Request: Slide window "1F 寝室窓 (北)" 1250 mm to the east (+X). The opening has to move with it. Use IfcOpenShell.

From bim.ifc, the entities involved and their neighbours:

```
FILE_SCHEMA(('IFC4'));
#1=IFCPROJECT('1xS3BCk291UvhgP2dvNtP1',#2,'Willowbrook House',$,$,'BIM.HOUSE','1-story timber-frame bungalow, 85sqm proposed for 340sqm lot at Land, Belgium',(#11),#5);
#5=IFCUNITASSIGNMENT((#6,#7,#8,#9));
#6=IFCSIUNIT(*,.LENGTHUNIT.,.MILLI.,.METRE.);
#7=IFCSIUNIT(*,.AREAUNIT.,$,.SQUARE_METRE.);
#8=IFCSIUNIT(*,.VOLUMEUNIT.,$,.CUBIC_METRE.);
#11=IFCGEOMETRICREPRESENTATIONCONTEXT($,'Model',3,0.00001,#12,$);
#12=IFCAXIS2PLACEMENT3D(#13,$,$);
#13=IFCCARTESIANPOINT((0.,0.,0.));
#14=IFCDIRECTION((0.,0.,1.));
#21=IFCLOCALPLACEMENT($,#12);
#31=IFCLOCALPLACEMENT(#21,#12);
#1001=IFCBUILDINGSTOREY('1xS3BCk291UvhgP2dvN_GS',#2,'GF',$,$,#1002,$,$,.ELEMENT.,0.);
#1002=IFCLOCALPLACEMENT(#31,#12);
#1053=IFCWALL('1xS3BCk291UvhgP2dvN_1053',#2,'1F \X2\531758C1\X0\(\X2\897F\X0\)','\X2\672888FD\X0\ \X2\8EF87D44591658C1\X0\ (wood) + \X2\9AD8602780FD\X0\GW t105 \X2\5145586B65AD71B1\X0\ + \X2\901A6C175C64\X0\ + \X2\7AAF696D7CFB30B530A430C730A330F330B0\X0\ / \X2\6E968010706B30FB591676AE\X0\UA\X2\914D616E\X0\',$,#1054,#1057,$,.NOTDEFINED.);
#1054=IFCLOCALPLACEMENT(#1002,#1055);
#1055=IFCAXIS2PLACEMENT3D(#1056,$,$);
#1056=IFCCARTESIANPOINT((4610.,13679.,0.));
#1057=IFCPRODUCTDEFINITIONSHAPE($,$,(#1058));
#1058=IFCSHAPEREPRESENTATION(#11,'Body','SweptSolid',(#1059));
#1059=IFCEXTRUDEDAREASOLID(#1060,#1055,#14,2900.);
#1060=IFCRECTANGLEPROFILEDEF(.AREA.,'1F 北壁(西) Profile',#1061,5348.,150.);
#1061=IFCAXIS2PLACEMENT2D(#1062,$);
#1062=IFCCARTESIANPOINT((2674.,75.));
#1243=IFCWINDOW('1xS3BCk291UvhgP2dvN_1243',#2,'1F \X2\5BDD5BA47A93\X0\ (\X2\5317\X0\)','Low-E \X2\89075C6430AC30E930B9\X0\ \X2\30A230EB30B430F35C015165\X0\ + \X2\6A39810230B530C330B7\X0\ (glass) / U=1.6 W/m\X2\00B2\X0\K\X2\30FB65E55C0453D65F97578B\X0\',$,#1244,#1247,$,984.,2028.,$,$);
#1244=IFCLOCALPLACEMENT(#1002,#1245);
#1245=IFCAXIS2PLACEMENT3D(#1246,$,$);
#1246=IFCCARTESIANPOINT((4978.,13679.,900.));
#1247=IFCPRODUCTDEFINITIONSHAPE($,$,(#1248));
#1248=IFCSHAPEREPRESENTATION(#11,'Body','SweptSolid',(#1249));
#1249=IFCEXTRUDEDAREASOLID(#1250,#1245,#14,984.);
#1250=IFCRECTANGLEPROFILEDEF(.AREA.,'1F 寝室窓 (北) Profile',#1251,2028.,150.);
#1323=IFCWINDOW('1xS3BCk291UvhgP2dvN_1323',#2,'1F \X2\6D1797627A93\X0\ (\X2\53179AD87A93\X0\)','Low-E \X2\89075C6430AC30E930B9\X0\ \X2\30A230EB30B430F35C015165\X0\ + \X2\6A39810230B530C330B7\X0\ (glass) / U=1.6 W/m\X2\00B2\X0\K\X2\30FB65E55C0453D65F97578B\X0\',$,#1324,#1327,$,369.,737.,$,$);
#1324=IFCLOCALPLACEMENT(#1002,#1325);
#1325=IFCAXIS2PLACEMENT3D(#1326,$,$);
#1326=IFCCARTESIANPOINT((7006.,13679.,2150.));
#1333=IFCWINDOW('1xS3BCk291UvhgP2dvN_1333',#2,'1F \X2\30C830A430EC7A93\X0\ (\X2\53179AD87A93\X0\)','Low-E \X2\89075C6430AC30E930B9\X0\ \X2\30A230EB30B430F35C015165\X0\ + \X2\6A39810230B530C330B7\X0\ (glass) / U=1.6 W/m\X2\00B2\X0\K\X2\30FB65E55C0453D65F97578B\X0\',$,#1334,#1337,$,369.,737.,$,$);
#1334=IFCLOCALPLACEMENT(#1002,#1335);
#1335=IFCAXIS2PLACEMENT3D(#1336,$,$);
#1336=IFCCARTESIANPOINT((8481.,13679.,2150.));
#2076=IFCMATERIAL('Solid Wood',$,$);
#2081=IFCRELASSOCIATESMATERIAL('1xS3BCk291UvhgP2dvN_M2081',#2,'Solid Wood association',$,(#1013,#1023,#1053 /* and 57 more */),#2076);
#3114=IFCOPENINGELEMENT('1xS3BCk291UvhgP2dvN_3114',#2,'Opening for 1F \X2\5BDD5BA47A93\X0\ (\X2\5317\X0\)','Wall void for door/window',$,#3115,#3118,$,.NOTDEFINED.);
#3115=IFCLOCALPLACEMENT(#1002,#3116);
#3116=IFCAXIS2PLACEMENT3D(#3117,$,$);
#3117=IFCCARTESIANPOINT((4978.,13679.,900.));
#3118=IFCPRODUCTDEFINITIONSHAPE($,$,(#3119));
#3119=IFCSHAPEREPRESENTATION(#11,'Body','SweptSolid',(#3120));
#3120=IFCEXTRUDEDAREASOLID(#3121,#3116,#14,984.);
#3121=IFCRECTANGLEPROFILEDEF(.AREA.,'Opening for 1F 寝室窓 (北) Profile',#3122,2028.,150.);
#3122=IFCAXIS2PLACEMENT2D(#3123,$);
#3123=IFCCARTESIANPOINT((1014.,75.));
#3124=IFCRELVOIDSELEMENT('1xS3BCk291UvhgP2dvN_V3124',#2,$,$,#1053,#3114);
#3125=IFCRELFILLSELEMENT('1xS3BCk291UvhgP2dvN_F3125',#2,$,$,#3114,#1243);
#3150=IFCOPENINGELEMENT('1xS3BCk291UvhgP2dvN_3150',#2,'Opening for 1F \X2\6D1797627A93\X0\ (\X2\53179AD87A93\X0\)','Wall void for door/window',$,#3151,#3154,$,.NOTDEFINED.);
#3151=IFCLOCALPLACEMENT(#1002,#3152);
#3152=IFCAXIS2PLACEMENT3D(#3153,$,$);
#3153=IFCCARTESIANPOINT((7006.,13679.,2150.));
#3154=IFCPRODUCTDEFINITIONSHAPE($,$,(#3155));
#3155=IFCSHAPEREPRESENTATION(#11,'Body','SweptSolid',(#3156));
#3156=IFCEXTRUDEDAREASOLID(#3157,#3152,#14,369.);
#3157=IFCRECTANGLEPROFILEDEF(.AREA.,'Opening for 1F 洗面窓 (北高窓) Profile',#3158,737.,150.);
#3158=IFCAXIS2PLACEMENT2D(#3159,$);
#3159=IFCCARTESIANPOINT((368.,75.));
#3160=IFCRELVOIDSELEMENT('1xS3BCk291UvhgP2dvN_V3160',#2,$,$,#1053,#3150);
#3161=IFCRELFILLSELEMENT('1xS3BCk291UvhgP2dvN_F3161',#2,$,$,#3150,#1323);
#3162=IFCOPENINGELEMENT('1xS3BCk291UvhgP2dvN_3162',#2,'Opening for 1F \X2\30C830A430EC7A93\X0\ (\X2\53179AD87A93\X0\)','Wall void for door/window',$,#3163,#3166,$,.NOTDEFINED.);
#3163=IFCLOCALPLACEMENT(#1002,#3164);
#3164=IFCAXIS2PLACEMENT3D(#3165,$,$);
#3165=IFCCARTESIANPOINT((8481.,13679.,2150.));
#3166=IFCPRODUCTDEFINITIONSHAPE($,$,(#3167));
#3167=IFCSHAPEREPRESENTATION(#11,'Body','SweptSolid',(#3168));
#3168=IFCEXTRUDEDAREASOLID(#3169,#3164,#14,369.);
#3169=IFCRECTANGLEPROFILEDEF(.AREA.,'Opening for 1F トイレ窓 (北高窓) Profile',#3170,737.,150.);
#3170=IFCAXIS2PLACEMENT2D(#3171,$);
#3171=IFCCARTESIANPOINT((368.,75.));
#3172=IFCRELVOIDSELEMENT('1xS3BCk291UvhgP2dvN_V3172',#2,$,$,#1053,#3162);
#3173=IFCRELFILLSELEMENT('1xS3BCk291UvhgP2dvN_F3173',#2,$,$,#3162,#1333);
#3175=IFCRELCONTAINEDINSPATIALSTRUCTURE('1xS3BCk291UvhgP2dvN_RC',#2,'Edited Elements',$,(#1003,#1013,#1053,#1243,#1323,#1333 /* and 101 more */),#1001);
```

```python
import ifcopenshell
import ifcopenshell.api.geometry
import ifcopenshell.util.placement

model = ifcopenshell.open("bim.ifc")

window = model.by_id(1243)
opening = window.FillsVoids[0].RelatingOpeningElement
wall = opening.VoidsElements[0].RelatingBuildingElement

wall_matrix = ifcopenshell.util.placement.get_local_placement(wall.ObjectPlacement)
shift = wall_matrix[:3, 0] * 1250.0
before = ifcopenshell.util.placement.get_local_placement(window.ObjectPlacement)[:3, 3].copy()

# The window is not placed relative to its opening, so move both.
for product in (opening, window):
    matrix = ifcopenshell.util.placement.get_local_placement(product.ObjectPlacement)
    matrix[:3, 3] += shift
    ifcopenshell.api.geometry.edit_object_placement(model, product=product, matrix=matrix, is_si=False)

after = ifcopenshell.util.placement.get_local_placement(window.ObjectPlacement)[:3, 3]
print("window moved by", (after - before).round(3) + 0.0)

model.write("bim_edited.ifc")
```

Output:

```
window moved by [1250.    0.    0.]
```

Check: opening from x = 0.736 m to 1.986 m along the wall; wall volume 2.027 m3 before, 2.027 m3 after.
